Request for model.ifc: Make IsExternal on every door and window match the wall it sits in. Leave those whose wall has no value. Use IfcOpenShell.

First a look at what the model holds.

```python
import ifcopenshell
import ifcopenshell.util.element

model = ifcopenshell.open("model.ifc")
print(model.schema)
seen = {}
for e in model.by_type("IfcDoor") + model.by_type("IfcWindow"):
    if not e.FillsVoids:
        continue
    host = e.FillsVoids[0].RelatingOpeningElement.VoidsElements[0].RelatingBuildingElement
    own = ifcopenshell.util.element.get_pset(e, f"Pset_{e.is_a()[3:].removesuffix('StandardCase')}Common", "IsExternal")
    wall = ifcopenshell.util.element.get_pset(host, "Pset_WallCommon", "IsExternal")
    seen[e.is_a(), own, wall] = seen.get((e.is_a(), own, wall), 0) + 1
for (cls, own, wall), count in sorted(seen.items(), key=str):
    print(count, cls, "IsExternal:", own, "| host wall:", wall)
```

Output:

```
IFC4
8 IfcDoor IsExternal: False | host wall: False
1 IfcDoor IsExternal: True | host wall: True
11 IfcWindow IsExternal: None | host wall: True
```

```python
import ifcopenshell
import ifcopenshell.api.pset
import ifcopenshell.util.element

model = ifcopenshell.open("model.ifc")

count = 0
for ifc_class, pset_name in (("IfcDoor", "Pset_DoorCommon"), ("IfcWindow", "Pset_WindowCommon")):
    for e in model.by_type(ifc_class):
        if not e.FillsVoids:
            continue
        host = e.FillsVoids[0].RelatingOpeningElement.VoidsElements[0].RelatingBuildingElement
        external = ifcopenshell.util.element.get_pset(host, "Pset_WallCommon", "IsExternal")
        if external is None or ifcopenshell.util.element.get_pset(e, pset_name, "IsExternal") == external:
            continue
        pset = ifcopenshell.api.pset.add_pset(model, product=e, name=pset_name)
        ifcopenshell.api.pset.edit_pset(model, pset=pset, properties={"IsExternal": external})
        count += 1

print(count, "updated")

model.write("model_v2.ifc")
```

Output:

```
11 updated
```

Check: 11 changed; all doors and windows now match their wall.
